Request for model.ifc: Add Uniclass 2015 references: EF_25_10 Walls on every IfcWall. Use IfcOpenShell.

First a look at what the model holds.

```python
import ifcopenshell

model = ifcopenshell.open("model.ifc")
print(model.schema)
print("classifications:", [c.Name for c in model.by_type("IfcClassification")])
for ifc_class in ("IfcDoor", "IfcRoof", "IfcStair", "IfcWall", "IfcWindow"):
    print(ifc_class, len(model.by_type(ifc_class)))
```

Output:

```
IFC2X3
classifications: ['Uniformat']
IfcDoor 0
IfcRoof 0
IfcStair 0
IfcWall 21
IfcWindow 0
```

```python
import ifcopenshell
import ifcopenshell.api.classification

model = ifcopenshell.open("model.ifc")

# IFC2X3 requires Source and Edition and has no link from the project to the system.
system = model.create_entity("IfcClassification", Source="NBS", Edition="2015", Name="Uniclass 2015")

codes = {
    "IfcWall": ("EF_25_10", "Walls"),
}
for ifc_class, (code, name) in codes.items():
    products = model.by_type(ifc_class)
    ifcopenshell.api.classification.add_reference(
        model, products=products, classification=system, identification=code, name=name
    )
    print(code, len(products))

model.write("model_rev.ifc")
```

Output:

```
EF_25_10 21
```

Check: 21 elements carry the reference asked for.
